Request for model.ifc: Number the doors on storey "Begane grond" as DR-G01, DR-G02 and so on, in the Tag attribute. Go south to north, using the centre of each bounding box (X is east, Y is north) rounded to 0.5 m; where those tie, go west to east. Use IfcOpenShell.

First a look at what the model holds.

```python
import ifcopenshell
import ifcopenshell.util.element
import ifcopenshell.util.placement

model = ifcopenshell.open("model.ifc")
print(model.schema)
storey = next(s for s in model.by_type("IfcBuildingStorey") if s.Name == "Begane grond")
doors = [e for e in ifcopenshell.util.element.get_decomposition(storey) if e.is_a("IfcDoor")]
for e in sorted(doors, key=lambda e: e.id()):
    origin = ifcopenshell.util.placement.get_local_placement(e.ObjectPlacement)[:3, 3]
    print(e.id(), e.Tag, e.Name, origin.round(2) + 0.0, sep=" | ")
```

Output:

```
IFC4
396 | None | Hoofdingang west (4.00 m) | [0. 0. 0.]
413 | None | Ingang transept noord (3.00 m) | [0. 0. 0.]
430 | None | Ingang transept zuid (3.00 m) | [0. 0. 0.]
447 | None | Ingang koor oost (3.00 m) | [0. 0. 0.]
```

```python
import ifcopenshell
import ifcopenshell.geom
import ifcopenshell.util.element
import ifcopenshell.util.shape

model = ifcopenshell.open("model.ifc")
settings = ifcopenshell.geom.settings()
settings.set("use-world-coords", True)


def centre(element):
    shape = ifcopenshell.geom.create_shape(settings, element)
    return ifcopenshell.util.shape.get_bbox_centroid(shape.geometry)


storey = next(s for s in model.by_type("IfcBuildingStorey") if s.Name == "Begane grond")
doors = [e for e in ifcopenshell.util.element.get_decomposition(storey) if e.is_a("IfcDoor")]

# Insertion points can sit at a corner or the storey origin, so sort by the geometry (in metres).
centres = {e: centre(e) for e in doors}
doors.sort(key=lambda e: (round(centres[e][1] / 0.5), centres[e][0]))

for i, e in enumerate(doors, start=1):
    number = f"DR-G{i:02d}"
    e.Tag = number
    print(e.id(), number)

model.write("model_edited.ifc")
```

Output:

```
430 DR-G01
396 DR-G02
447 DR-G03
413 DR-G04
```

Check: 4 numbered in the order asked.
